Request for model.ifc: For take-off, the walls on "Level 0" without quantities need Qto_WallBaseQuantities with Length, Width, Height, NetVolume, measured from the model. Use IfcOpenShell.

First a look at what the model holds.

```python
import ifcopenshell
import ifcopenshell.util.element
import ifcopenshell.util.unit

model = ifcopenshell.open("model.ifc")
print(model.schema)
for unit_type in ("LENGTHUNIT", "AREAUNIT", "VOLUMEUNIT"):
    print(unit_type, ifcopenshell.util.unit.calculate_unit_scale(model, unit_type))
storey = next(s for s in model.by_type("IfcBuildingStorey") if s.Name == "Level 0")
walls = [e for e in ifcopenshell.util.element.get_decomposition(storey) if e.is_a("IfcWall")]
for e in sorted(walls, key=lambda e: e.id()):
    print(e.id(), e.is_a(), e.Name, list(ifcopenshell.util.element.get_psets(e, qtos_only=True)), sep=" | ")
```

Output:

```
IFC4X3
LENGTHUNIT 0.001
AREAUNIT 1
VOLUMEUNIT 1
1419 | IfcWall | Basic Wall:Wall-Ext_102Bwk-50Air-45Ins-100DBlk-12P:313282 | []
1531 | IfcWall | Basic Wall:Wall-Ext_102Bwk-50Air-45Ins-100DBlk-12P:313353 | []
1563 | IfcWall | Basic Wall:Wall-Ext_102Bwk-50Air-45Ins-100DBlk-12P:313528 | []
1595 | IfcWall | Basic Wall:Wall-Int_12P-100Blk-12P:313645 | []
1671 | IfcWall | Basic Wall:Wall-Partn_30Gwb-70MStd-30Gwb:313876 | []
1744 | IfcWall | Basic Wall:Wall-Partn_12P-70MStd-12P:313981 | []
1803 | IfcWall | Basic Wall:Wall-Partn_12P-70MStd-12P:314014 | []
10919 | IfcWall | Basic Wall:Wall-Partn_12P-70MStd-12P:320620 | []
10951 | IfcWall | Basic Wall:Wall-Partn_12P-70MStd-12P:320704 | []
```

```python
import ifcopenshell
import ifcopenshell.api.pset
import ifcopenshell.geom
import ifcopenshell.util.element
import ifcopenshell.util.shape
import ifcopenshell.util.unit

model = ifcopenshell.open("model.ifc")
unit_scale = ifcopenshell.util.unit.calculate_unit_scale(model)
volume_scale = ifcopenshell.util.unit.calculate_unit_scale(model, "VOLUMEUNIT")
settings = ifcopenshell.geom.settings()

storey = next(s for s in model.by_type("IfcBuildingStorey") if s.Name == "Level 0")
walls = [e for e in ifcopenshell.util.element.get_decomposition(storey) if e.is_a("IfcWall")]

for e in sorted(walls, key=lambda e: e.id()):
    if ifcopenshell.util.element.get_psets(e, qtos_only=True, should_inherit=False):
        continue
    # Geometry comes back in metres, in the element's own axes.
    shape = ifcopenshell.geom.create_shape(settings, e)
    values = {
        "Length": ifcopenshell.util.shape.get_x(shape.geometry) / unit_scale,
        "Width": ifcopenshell.util.shape.get_y(shape.geometry) / unit_scale,
        "Height": ifcopenshell.util.shape.get_z(shape.geometry) / unit_scale,
        "NetVolume": ifcopenshell.util.shape.get_volume(shape.geometry) / volume_scale,
    }
    qto = ifcopenshell.api.pset.add_qto(model, product=e, name="Qto_WallBaseQuantities")
    ifcopenshell.api.pset.edit_qto(model, qto=qto, properties=values)
    print(e.id(), {k: round(v, 3) for k, v in values.items()})

model.write("model-out.ifc")
```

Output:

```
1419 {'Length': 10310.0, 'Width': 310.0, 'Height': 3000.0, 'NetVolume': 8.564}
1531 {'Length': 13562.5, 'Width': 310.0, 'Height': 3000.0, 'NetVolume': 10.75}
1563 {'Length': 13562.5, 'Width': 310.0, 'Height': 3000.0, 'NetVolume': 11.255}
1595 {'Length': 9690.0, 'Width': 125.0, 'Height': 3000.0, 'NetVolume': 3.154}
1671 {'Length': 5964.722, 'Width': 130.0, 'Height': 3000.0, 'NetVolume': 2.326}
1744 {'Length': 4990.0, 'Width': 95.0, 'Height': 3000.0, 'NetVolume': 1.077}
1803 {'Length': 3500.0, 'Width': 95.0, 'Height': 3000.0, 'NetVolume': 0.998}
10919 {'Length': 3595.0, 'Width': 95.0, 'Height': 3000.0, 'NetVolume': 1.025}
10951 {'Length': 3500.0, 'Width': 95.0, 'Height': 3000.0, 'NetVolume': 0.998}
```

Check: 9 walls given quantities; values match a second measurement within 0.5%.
